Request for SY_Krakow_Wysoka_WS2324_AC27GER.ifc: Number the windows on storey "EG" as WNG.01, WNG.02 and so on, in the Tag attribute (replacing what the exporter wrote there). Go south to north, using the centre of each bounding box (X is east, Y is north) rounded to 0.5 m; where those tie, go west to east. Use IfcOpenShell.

First a look at what the model holds.

```python
import ifcopenshell
import ifcopenshell.util.element
import ifcopenshell.util.placement

model = ifcopenshell.open("SY_Krakow_Wysoka_WS2324_AC27GER.ifc")
print(model.schema)
storey = next(s for s in model.by_type("IfcBuildingStorey") if s.Name == "EG")
windows = [e for e in ifcopenshell.util.element.get_decomposition(storey) if e.is_a("IfcWindow")]
for e in sorted(windows, key=lambda e: e.id()):
    origin = ifcopenshell.util.placement.get_local_placement(e.ObjectPlacement)[:3, 3]
    print(e.id(), e.Tag, e.Name, origin.round(2) + 0.0, sep=" | ")
```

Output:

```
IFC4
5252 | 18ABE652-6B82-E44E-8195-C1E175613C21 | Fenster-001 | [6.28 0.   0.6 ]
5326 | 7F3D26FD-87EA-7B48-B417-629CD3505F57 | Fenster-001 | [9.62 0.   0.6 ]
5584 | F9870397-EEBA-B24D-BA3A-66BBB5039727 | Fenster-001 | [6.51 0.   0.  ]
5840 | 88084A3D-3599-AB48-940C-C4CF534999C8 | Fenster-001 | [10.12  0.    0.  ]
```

```python
import ifcopenshell
import ifcopenshell.geom
import ifcopenshell.util.element
import ifcopenshell.util.shape

model = ifcopenshell.open("SY_Krakow_Wysoka_WS2324_AC27GER.ifc")
settings = ifcopenshell.geom.settings()
settings.set("use-world-coords", True)


def centre(element):
    shape = ifcopenshell.geom.create_shape(settings, element)
    return ifcopenshell.util.shape.get_bbox_centroid(shape.geometry)


storey = next(s for s in model.by_type("IfcBuildingStorey") if s.Name == "EG")
windows = [e for e in ifcopenshell.util.element.get_decomposition(storey) if e.is_a("IfcWindow")]

# Insertion points can sit at a corner or the storey origin, so sort by the geometry (in metres).
centres = {e: centre(e) for e in windows}
windows.sort(key=lambda e: (round(centres[e][1] / 0.5), centres[e][0]))

for i, e in enumerate(windows, start=1):
    number = f"WNG.{i:02d}"
    e.Tag = number
    print(e.id(), number)

model.write("SY_Krakow_Wysoka_WS2324_AC27GER_edited.ifc")
```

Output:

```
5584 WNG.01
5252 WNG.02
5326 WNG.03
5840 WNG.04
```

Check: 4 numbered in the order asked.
